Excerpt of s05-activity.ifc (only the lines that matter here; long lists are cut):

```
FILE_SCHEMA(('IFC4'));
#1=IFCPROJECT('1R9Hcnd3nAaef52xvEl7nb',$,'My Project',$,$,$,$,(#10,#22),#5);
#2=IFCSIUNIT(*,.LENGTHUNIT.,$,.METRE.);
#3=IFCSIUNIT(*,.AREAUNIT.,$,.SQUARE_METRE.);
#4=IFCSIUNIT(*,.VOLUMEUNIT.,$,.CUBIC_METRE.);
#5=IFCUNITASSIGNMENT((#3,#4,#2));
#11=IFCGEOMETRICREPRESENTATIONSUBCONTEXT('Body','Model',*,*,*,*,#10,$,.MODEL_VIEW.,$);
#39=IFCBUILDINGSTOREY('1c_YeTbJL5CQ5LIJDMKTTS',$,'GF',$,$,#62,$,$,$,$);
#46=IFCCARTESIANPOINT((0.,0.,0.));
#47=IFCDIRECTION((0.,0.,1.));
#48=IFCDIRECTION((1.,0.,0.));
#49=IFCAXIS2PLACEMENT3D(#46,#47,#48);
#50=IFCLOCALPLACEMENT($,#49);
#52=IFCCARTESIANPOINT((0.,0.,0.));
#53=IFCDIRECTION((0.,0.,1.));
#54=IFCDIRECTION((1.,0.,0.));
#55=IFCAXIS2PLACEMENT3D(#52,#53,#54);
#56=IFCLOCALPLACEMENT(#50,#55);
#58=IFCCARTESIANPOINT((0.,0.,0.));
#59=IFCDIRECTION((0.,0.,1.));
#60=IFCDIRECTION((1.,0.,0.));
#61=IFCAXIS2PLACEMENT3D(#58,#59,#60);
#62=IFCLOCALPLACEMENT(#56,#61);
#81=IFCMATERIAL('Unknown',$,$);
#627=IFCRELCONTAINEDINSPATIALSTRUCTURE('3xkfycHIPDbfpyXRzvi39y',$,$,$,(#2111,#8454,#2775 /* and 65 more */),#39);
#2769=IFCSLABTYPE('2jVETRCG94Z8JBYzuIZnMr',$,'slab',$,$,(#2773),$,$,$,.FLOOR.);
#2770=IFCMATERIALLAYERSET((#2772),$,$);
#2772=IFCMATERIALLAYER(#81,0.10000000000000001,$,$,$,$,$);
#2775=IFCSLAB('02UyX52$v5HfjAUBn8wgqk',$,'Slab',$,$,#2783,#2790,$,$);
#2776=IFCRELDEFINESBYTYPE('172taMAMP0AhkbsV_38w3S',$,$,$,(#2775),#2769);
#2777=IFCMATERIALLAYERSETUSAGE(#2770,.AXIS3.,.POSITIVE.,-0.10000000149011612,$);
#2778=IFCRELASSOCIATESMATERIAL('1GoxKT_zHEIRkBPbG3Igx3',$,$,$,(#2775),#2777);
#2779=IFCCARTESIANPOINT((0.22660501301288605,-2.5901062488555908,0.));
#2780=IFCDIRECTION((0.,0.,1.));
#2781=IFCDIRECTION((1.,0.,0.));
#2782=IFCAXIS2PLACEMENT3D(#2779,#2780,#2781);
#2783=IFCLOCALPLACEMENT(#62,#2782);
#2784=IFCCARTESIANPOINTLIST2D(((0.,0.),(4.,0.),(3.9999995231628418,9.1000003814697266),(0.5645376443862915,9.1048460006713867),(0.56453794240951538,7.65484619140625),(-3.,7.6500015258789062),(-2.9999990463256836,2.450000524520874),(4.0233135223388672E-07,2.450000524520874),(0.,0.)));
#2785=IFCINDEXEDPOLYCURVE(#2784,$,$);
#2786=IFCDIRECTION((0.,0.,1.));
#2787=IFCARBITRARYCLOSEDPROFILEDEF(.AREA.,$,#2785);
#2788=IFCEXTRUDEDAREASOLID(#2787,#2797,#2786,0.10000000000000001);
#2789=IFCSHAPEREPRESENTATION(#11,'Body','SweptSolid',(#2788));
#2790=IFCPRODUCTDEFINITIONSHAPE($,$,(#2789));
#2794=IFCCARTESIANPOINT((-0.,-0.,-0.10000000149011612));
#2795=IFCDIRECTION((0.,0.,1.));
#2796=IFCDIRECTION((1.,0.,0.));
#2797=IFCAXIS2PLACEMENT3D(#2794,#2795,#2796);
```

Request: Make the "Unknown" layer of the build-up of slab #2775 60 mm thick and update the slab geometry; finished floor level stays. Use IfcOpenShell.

```python
import ifcopenshell
import ifcopenshell.util.element
import ifcopenshell.util.representation

model = ifcopenshell.open("s05-activity.ifc")

layer_set = model.by_id(2770)
layer = next(l for l in layer_set.MaterialLayers if l.Material and l.Material.Name == "Unknown")
change = 0.06 - layer.LayerThickness
layer.LayerThickness += change

# Geometry does not follow the layer set by itself.
slabs = [e for e in ifcopenshell.util.element.get_elements_by_material(model, layer_set) if e.is_a("IfcSlab")]
for slab in sorted(slabs, key=lambda e: e.id()):
    body = ifcopenshell.util.representation.get_representation(slab, "Model", "Body")
    solid = body.Items[0]
    old_depth = solid.Depth
    solid.Depth += change
    # Extruded upwards: lower the start of the extrusion so the top stays.
    x, y, z = solid.Position.Location.Coordinates
    solid.Position.Location = model.createIfcCartesianPoint((x, y, z - change))
    print(slab.id(), f"{old_depth:g} -> {solid.Depth:g}")

# The layers are counted up from the underside, which has moved.
for usage in {ifcopenshell.util.element.get_material(slab) for slab in slabs}:
    usage.OffsetFromReferenceLine -= change

model.write("s05-activity_v2.ifc")
```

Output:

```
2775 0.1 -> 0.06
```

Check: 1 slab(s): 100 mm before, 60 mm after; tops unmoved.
